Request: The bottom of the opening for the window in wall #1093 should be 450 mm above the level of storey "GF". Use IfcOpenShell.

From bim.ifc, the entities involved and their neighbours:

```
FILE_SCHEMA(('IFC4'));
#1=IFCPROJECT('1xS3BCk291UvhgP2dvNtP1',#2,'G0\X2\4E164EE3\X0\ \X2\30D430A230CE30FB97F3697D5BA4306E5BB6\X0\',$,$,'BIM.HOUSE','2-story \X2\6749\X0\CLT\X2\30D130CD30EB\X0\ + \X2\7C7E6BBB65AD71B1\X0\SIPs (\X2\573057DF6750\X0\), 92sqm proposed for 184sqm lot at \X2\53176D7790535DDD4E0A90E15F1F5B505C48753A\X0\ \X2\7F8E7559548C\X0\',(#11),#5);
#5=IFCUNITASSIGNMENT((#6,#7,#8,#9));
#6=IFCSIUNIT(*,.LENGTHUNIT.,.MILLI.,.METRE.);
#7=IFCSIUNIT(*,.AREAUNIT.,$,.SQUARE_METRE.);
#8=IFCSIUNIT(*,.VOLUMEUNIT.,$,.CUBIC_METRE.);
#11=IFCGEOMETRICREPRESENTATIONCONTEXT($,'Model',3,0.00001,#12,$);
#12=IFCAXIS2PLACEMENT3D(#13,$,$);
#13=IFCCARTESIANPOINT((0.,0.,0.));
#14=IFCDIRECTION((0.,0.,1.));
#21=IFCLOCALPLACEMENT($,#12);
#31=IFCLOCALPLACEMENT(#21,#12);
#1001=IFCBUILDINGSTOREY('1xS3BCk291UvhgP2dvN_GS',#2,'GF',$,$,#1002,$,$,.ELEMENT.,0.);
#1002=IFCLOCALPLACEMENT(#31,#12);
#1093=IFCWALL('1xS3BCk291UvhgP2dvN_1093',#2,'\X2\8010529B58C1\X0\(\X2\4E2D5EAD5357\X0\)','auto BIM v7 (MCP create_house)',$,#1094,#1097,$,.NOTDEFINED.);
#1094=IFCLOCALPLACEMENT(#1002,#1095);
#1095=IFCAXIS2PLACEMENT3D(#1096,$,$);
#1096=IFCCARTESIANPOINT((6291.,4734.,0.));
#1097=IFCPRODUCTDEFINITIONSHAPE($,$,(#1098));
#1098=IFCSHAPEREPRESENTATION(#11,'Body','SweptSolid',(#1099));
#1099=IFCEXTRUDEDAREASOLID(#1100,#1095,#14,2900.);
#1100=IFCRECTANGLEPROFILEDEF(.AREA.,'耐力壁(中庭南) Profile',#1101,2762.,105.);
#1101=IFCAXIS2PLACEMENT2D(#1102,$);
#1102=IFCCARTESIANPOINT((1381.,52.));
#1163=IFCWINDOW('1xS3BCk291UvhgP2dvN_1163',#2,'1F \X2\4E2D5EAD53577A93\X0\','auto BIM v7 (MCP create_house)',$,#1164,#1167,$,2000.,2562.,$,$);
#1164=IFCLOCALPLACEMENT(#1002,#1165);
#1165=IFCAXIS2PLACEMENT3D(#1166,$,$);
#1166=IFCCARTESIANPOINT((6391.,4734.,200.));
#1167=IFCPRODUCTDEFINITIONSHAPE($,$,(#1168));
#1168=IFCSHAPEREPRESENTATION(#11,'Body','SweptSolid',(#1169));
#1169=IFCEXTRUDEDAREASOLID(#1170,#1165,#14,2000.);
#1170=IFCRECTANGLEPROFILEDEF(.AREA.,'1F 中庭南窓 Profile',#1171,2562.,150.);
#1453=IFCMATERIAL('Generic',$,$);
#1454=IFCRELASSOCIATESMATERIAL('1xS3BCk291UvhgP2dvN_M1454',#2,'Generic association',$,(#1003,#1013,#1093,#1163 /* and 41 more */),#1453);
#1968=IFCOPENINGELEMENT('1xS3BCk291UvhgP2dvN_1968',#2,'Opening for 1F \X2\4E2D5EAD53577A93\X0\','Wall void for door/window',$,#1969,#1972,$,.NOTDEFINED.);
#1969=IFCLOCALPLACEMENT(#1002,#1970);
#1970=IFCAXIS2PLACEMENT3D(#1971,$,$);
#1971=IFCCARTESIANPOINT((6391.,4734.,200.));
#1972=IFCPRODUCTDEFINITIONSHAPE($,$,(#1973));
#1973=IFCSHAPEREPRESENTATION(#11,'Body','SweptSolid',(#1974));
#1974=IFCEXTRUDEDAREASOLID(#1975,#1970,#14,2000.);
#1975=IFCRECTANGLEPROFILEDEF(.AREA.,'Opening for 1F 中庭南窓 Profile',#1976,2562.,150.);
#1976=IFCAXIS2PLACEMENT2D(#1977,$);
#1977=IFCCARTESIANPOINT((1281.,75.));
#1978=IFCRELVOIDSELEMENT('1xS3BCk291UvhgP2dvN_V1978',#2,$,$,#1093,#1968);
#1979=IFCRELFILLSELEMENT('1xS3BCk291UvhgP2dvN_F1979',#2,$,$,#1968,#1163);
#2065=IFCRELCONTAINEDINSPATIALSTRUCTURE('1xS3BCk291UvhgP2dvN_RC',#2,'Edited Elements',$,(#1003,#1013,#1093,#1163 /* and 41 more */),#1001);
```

```python
import numpy as np
import ifcopenshell
import ifcopenshell.api.geometry
import ifcopenshell.geom
import ifcopenshell.util.element
import ifcopenshell.util.placement
import ifcopenshell.util.shape
import ifcopenshell.util.unit

model = ifcopenshell.open("bim.ifc")
unit_scale = ifcopenshell.util.unit.calculate_unit_scale(model)

window = model.by_guid("1xS3BCk291UvhgP2dvN_1163")
opening = window.FillsVoids[0].RelatingOpeningElement
storey = ifcopenshell.util.element.get_container(window, ifc_class="IfcBuildingStorey")
level = ifcopenshell.util.placement.get_local_placement(storey.ObjectPlacement)[2, 3]

# The opening's origin need not be at the sill, so measure its lowest point.
shape = ifcopenshell.geom.create_shape(ifcopenshell.geom.settings(), opening)
bottom = ifcopenshell.util.shape.get_shape_bottom_elevation(shape, shape.geometry) / unit_scale
dz = level + 0.45 / unit_scale - bottom

shift = np.array([0.0, 0.0, dz])
# The window is not placed relative to its opening, so move both.
for product in (opening, window):
    matrix = ifcopenshell.util.placement.get_local_placement(product.ObjectPlacement)
    matrix[:3, 3] += shift
    ifcopenshell.api.geometry.edit_object_placement(model, product=product, matrix=matrix, is_si=False)

print(f"moved by {dz * unit_scale:+.3f} m")

model.write("bim_edited.ifc")
```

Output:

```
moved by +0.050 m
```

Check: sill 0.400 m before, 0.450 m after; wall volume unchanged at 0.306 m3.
